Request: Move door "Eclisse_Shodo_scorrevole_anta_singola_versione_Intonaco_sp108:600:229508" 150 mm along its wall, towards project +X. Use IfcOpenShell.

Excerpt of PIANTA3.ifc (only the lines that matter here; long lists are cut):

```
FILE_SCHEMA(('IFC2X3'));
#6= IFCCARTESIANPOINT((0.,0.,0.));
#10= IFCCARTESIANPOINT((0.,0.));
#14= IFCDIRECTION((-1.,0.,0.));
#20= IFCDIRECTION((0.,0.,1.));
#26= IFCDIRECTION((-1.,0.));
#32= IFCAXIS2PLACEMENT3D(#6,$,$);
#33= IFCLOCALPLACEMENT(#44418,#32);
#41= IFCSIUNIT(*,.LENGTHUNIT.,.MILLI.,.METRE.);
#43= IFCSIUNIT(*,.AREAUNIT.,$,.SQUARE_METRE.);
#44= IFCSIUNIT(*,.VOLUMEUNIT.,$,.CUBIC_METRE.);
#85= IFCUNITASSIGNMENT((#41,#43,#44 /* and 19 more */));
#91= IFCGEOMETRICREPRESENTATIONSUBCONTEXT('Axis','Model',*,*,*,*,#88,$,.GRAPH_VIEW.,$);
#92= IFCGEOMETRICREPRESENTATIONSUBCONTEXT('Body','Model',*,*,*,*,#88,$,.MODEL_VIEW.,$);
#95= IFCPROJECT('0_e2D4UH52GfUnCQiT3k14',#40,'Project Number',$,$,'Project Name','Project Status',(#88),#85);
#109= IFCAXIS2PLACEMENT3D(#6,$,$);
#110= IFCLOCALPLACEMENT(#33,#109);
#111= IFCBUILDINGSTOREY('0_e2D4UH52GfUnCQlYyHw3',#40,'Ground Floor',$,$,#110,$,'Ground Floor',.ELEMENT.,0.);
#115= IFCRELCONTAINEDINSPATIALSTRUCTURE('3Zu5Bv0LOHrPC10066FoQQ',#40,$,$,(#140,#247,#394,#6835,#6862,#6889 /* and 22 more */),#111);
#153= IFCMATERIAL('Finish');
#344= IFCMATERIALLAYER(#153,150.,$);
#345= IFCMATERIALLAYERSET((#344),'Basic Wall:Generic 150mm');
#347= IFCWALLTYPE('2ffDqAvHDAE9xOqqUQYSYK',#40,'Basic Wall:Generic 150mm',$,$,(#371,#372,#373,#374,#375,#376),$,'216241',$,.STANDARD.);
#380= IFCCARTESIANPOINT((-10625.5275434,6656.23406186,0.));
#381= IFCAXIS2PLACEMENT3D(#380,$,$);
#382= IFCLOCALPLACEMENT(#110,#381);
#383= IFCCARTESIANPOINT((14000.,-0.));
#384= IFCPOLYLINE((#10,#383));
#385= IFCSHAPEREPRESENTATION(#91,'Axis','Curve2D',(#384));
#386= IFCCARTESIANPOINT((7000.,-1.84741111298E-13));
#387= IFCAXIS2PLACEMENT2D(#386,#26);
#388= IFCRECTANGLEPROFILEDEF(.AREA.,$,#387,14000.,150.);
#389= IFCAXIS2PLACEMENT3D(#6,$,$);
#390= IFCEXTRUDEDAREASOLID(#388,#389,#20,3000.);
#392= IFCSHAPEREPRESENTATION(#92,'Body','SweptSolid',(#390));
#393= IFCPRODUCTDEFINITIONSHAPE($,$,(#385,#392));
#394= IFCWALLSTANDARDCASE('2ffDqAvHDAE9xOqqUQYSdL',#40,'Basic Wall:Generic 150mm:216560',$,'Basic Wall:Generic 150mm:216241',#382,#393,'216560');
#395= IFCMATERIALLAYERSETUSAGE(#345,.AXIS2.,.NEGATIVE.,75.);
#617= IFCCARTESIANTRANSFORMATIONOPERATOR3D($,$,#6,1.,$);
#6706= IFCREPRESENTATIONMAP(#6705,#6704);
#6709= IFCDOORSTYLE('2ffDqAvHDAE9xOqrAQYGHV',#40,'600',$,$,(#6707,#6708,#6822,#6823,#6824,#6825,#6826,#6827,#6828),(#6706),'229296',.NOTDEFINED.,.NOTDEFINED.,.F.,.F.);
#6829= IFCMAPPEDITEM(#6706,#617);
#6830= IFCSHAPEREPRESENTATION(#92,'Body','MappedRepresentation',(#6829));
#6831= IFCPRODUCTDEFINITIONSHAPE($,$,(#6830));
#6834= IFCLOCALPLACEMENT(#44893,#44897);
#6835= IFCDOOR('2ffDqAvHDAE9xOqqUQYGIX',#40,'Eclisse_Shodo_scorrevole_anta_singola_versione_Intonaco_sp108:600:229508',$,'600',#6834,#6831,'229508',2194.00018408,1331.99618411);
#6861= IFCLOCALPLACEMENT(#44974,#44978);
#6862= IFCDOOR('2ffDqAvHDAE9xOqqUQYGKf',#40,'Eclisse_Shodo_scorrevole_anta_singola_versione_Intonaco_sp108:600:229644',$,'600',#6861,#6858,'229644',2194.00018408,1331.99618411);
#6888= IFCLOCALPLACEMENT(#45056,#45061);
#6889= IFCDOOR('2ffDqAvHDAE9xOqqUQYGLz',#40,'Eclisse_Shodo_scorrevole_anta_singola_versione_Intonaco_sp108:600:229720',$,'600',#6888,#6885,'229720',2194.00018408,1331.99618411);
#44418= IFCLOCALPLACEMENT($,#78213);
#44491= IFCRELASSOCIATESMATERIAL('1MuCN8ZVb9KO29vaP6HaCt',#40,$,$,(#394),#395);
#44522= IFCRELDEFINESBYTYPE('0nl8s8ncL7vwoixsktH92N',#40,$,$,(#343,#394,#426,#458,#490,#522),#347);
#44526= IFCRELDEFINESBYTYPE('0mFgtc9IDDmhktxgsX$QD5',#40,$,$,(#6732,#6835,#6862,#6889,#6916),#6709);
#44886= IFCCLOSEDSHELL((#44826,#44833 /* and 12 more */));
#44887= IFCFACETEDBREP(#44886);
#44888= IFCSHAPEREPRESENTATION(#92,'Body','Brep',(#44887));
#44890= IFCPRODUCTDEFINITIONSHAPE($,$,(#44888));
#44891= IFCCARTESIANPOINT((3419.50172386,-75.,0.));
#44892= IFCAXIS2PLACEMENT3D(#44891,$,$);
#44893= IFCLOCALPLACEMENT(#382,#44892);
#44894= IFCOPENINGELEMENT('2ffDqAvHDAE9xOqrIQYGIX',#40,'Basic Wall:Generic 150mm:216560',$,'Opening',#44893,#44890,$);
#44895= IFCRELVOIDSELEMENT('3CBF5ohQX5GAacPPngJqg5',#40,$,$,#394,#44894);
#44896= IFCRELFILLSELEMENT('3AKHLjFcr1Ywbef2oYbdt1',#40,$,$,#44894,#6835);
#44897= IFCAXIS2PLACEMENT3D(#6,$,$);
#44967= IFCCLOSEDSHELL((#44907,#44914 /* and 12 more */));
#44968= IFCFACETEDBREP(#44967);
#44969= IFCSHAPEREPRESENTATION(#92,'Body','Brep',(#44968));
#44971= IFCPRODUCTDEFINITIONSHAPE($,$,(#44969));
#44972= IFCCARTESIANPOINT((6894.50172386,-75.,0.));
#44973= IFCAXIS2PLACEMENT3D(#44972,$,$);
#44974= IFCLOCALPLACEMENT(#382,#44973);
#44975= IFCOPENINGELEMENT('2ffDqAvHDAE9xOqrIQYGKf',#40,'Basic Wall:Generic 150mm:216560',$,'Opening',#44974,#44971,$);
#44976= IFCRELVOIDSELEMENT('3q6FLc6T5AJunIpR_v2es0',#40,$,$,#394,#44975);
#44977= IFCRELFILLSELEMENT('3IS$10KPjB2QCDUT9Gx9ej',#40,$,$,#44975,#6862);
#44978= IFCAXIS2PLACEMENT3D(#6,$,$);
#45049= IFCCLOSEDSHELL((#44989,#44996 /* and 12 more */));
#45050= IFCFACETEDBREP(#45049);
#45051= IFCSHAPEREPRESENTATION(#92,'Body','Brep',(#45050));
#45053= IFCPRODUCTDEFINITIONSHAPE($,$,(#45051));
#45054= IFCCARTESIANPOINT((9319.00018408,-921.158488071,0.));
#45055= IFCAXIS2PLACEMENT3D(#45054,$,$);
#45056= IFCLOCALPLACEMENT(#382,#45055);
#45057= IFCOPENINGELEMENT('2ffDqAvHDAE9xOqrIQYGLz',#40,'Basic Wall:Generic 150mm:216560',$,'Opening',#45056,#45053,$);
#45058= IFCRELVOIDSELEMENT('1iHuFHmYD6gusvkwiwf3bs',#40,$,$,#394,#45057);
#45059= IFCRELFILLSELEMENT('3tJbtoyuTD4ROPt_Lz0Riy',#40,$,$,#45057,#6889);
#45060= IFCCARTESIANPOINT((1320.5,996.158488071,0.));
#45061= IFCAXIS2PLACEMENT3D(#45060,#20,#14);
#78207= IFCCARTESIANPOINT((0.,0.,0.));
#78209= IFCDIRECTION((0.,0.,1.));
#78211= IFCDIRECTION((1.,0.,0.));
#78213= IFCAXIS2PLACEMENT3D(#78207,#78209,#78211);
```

```python
import ifcopenshell
import ifcopenshell.api.geometry
import ifcopenshell.util.placement

model = ifcopenshell.open("PIANTA3.ifc")

door = model.by_guid("2ffDqAvHDAE9xOqqUQYGIX")
opening = door.FillsVoids[0].RelatingOpeningElement
wall = opening.VoidsElements[0].RelatingBuildingElement

wall_matrix = ifcopenshell.util.placement.get_local_placement(wall.ObjectPlacement)
shift = wall_matrix[:3, 0] * 150.0
before = ifcopenshell.util.placement.get_local_placement(door.ObjectPlacement)[:3, 3].copy()

# The door is placed relative to its opening, so it follows when the opening moves.
matrix = ifcopenshell.util.placement.get_local_placement(opening.ObjectPlacement)
matrix[:3, 3] += shift
ifcopenshell.api.geometry.edit_object_placement(
    model, product=opening, matrix=matrix, is_si=False, should_transform_children=True
)

after = ifcopenshell.util.placement.get_local_placement(door.ObjectPlacement)[:3, 3]
print("door moved by", (after - before).round(3) + 0.0)

model.write("PIANTA3_updated.ifc")
```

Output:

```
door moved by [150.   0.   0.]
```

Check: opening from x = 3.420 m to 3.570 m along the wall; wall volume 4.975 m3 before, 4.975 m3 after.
